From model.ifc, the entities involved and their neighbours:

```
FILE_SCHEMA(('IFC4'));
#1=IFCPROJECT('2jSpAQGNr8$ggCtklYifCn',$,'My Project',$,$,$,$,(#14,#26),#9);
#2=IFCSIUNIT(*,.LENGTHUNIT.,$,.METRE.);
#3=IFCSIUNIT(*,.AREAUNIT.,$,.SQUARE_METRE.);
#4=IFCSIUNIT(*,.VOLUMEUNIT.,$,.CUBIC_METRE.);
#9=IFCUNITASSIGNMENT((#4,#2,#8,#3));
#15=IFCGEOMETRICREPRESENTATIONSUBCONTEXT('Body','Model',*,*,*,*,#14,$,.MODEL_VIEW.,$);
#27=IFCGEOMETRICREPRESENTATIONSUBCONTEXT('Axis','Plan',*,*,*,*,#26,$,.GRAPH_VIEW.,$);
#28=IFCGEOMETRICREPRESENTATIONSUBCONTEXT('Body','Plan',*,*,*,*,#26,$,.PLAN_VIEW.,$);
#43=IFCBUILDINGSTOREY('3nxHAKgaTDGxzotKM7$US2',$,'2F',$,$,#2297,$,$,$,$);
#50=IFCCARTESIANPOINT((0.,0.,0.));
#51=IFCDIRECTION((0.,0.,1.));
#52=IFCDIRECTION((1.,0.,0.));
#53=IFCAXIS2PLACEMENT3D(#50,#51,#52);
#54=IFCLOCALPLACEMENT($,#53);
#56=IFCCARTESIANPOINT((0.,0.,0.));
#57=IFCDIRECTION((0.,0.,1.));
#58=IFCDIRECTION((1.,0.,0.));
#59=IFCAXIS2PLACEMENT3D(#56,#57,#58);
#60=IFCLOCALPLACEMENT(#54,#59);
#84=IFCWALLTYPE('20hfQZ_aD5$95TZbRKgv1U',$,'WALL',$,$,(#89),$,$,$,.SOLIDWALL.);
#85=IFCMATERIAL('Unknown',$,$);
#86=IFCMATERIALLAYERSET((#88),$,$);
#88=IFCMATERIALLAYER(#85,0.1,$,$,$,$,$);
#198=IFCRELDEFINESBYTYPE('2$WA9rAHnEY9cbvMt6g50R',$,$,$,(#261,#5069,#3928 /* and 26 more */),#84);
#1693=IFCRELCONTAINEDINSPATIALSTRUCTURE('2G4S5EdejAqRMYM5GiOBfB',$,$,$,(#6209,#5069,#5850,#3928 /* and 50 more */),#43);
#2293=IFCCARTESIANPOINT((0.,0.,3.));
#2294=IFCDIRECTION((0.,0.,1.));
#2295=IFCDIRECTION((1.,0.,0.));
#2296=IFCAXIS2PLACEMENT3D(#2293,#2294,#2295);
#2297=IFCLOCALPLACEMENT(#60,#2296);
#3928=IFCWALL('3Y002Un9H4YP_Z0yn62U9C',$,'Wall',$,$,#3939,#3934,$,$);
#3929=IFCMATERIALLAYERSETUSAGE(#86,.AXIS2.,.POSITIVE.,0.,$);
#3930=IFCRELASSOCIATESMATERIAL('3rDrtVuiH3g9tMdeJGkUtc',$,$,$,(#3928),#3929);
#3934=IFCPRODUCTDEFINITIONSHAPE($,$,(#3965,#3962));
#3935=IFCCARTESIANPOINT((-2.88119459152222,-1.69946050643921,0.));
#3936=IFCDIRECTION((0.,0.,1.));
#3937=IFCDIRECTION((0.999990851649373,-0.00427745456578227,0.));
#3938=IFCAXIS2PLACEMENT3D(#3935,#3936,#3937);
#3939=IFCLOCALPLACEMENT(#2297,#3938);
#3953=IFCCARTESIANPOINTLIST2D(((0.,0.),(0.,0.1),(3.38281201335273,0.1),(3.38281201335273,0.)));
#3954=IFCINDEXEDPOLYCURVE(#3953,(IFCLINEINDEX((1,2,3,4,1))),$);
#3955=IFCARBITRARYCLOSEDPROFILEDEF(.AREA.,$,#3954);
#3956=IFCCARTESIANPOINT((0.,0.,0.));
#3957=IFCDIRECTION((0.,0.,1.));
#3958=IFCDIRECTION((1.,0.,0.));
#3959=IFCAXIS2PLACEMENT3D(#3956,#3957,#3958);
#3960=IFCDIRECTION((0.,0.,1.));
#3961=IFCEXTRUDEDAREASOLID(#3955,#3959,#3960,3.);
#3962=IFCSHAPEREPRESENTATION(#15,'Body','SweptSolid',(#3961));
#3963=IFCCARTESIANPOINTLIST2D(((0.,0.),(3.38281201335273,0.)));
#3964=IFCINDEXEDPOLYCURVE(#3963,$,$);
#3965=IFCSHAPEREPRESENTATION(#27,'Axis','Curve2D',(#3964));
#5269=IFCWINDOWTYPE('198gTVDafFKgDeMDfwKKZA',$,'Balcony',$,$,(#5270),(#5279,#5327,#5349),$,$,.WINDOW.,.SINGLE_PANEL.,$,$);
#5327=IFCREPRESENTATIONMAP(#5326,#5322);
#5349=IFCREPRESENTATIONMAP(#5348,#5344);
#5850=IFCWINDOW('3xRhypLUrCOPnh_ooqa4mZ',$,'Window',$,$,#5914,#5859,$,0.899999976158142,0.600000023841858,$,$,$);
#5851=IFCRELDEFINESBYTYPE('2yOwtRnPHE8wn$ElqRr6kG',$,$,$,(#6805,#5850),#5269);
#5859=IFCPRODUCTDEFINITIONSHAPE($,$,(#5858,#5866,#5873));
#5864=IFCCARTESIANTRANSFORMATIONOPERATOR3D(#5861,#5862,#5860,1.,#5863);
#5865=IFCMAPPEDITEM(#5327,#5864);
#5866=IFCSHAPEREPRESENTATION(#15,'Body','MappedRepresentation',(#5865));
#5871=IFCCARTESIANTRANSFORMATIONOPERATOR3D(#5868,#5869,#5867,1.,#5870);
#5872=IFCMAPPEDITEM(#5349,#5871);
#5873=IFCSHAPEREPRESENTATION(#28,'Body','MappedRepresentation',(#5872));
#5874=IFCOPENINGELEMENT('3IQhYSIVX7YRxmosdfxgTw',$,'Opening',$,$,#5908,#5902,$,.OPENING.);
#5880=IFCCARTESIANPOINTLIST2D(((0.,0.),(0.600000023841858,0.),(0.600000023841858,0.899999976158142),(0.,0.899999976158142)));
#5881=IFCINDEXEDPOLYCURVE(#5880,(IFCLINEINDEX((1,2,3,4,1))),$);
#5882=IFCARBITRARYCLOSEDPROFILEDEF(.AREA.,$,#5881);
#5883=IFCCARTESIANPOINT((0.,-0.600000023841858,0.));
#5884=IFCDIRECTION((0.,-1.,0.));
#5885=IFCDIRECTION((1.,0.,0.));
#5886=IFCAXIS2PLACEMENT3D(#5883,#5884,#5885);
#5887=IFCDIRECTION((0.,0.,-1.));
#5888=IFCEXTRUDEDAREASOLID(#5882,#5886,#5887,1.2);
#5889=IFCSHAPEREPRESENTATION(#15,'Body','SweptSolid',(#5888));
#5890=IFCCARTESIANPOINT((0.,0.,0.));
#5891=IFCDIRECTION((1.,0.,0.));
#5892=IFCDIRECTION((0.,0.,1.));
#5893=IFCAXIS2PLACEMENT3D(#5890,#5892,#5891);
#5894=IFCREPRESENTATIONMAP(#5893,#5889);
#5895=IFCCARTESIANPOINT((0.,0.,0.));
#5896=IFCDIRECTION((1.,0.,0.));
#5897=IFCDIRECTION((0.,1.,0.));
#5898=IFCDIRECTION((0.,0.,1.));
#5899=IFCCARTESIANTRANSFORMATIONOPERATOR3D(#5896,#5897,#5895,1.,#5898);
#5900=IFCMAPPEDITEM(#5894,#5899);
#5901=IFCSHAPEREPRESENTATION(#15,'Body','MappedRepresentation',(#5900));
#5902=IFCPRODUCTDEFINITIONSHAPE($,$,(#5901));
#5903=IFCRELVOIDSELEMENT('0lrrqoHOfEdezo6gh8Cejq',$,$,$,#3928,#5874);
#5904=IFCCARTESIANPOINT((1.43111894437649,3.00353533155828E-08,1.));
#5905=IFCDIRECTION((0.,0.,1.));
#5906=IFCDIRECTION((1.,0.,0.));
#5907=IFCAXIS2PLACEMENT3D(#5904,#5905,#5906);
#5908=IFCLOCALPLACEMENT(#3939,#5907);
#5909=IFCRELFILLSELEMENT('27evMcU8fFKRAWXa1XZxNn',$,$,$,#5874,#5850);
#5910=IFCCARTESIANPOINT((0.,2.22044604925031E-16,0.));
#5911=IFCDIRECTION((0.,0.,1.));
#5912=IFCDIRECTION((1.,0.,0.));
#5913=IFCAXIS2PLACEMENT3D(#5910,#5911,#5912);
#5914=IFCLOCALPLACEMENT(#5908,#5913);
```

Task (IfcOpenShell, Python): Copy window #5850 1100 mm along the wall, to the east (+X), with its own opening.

```python
import ifcopenshell
import ifcopenshell.api.feature
import ifcopenshell.api.geometry
import ifcopenshell.api.root
import ifcopenshell.geom
import ifcopenshell.util.element
import ifcopenshell.util.placement
import ifcopenshell.util.shape
import ifcopenshell.util.unit

model = ifcopenshell.open("model.ifc")
unit_scale = ifcopenshell.util.unit.calculate_unit_scale(model)
settings = ifcopenshell.geom.settings()


def volume(element):
    """Net volume in cubic metres, openings subtracted."""
    shape = ifcopenshell.geom.create_shape(settings, element)
    return ifcopenshell.util.shape.get_volume(shape.geometry)


window = model.by_guid("3xRhypLUrCOPnh_ooqa4mZ")
opening = window.FillsVoids[0].RelatingOpeningElement
wall = opening.VoidsElements[0].RelatingBuildingElement
before = volume(wall)
shift = ifcopenshell.util.placement.get_local_placement(wall.ObjectPlacement)[:3, 0] * 1.1 / unit_scale

# copy_class copies the void relationship, type, container and properties, but no geometry.
new_opening = ifcopenshell.api.root.copy_class(model, product=opening)
new_opening.Representation = ifcopenshell.util.element.copy_deep(
    model, opening.Representation, exclude=["IfcGeometricRepresentationContext", "IfcRepresentationMap"]
)
new_window = ifcopenshell.api.root.copy_class(model, product=window)
new_window.Representation = ifcopenshell.util.element.copy_deep(
    model, window.Representation, exclude=["IfcGeometricRepresentationContext", "IfcRepresentationMap"]
)
ifcopenshell.api.feature.add_filling(model, opening=new_opening, element=new_window)

for old, new in ((opening, new_opening), (window, new_window)):
    matrix = ifcopenshell.util.placement.get_local_placement(old.ObjectPlacement)
    matrix[:3, 3] += shift
    ifcopenshell.api.geometry.edit_object_placement(model, product=new, matrix=matrix, is_si=False)

after = volume(wall)

print(f"wall volume {before:.3f} -> {after:.3f} m3")

model.write("model_v2.ifc")
```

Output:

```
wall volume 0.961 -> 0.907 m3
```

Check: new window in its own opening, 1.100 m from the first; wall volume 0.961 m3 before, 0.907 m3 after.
